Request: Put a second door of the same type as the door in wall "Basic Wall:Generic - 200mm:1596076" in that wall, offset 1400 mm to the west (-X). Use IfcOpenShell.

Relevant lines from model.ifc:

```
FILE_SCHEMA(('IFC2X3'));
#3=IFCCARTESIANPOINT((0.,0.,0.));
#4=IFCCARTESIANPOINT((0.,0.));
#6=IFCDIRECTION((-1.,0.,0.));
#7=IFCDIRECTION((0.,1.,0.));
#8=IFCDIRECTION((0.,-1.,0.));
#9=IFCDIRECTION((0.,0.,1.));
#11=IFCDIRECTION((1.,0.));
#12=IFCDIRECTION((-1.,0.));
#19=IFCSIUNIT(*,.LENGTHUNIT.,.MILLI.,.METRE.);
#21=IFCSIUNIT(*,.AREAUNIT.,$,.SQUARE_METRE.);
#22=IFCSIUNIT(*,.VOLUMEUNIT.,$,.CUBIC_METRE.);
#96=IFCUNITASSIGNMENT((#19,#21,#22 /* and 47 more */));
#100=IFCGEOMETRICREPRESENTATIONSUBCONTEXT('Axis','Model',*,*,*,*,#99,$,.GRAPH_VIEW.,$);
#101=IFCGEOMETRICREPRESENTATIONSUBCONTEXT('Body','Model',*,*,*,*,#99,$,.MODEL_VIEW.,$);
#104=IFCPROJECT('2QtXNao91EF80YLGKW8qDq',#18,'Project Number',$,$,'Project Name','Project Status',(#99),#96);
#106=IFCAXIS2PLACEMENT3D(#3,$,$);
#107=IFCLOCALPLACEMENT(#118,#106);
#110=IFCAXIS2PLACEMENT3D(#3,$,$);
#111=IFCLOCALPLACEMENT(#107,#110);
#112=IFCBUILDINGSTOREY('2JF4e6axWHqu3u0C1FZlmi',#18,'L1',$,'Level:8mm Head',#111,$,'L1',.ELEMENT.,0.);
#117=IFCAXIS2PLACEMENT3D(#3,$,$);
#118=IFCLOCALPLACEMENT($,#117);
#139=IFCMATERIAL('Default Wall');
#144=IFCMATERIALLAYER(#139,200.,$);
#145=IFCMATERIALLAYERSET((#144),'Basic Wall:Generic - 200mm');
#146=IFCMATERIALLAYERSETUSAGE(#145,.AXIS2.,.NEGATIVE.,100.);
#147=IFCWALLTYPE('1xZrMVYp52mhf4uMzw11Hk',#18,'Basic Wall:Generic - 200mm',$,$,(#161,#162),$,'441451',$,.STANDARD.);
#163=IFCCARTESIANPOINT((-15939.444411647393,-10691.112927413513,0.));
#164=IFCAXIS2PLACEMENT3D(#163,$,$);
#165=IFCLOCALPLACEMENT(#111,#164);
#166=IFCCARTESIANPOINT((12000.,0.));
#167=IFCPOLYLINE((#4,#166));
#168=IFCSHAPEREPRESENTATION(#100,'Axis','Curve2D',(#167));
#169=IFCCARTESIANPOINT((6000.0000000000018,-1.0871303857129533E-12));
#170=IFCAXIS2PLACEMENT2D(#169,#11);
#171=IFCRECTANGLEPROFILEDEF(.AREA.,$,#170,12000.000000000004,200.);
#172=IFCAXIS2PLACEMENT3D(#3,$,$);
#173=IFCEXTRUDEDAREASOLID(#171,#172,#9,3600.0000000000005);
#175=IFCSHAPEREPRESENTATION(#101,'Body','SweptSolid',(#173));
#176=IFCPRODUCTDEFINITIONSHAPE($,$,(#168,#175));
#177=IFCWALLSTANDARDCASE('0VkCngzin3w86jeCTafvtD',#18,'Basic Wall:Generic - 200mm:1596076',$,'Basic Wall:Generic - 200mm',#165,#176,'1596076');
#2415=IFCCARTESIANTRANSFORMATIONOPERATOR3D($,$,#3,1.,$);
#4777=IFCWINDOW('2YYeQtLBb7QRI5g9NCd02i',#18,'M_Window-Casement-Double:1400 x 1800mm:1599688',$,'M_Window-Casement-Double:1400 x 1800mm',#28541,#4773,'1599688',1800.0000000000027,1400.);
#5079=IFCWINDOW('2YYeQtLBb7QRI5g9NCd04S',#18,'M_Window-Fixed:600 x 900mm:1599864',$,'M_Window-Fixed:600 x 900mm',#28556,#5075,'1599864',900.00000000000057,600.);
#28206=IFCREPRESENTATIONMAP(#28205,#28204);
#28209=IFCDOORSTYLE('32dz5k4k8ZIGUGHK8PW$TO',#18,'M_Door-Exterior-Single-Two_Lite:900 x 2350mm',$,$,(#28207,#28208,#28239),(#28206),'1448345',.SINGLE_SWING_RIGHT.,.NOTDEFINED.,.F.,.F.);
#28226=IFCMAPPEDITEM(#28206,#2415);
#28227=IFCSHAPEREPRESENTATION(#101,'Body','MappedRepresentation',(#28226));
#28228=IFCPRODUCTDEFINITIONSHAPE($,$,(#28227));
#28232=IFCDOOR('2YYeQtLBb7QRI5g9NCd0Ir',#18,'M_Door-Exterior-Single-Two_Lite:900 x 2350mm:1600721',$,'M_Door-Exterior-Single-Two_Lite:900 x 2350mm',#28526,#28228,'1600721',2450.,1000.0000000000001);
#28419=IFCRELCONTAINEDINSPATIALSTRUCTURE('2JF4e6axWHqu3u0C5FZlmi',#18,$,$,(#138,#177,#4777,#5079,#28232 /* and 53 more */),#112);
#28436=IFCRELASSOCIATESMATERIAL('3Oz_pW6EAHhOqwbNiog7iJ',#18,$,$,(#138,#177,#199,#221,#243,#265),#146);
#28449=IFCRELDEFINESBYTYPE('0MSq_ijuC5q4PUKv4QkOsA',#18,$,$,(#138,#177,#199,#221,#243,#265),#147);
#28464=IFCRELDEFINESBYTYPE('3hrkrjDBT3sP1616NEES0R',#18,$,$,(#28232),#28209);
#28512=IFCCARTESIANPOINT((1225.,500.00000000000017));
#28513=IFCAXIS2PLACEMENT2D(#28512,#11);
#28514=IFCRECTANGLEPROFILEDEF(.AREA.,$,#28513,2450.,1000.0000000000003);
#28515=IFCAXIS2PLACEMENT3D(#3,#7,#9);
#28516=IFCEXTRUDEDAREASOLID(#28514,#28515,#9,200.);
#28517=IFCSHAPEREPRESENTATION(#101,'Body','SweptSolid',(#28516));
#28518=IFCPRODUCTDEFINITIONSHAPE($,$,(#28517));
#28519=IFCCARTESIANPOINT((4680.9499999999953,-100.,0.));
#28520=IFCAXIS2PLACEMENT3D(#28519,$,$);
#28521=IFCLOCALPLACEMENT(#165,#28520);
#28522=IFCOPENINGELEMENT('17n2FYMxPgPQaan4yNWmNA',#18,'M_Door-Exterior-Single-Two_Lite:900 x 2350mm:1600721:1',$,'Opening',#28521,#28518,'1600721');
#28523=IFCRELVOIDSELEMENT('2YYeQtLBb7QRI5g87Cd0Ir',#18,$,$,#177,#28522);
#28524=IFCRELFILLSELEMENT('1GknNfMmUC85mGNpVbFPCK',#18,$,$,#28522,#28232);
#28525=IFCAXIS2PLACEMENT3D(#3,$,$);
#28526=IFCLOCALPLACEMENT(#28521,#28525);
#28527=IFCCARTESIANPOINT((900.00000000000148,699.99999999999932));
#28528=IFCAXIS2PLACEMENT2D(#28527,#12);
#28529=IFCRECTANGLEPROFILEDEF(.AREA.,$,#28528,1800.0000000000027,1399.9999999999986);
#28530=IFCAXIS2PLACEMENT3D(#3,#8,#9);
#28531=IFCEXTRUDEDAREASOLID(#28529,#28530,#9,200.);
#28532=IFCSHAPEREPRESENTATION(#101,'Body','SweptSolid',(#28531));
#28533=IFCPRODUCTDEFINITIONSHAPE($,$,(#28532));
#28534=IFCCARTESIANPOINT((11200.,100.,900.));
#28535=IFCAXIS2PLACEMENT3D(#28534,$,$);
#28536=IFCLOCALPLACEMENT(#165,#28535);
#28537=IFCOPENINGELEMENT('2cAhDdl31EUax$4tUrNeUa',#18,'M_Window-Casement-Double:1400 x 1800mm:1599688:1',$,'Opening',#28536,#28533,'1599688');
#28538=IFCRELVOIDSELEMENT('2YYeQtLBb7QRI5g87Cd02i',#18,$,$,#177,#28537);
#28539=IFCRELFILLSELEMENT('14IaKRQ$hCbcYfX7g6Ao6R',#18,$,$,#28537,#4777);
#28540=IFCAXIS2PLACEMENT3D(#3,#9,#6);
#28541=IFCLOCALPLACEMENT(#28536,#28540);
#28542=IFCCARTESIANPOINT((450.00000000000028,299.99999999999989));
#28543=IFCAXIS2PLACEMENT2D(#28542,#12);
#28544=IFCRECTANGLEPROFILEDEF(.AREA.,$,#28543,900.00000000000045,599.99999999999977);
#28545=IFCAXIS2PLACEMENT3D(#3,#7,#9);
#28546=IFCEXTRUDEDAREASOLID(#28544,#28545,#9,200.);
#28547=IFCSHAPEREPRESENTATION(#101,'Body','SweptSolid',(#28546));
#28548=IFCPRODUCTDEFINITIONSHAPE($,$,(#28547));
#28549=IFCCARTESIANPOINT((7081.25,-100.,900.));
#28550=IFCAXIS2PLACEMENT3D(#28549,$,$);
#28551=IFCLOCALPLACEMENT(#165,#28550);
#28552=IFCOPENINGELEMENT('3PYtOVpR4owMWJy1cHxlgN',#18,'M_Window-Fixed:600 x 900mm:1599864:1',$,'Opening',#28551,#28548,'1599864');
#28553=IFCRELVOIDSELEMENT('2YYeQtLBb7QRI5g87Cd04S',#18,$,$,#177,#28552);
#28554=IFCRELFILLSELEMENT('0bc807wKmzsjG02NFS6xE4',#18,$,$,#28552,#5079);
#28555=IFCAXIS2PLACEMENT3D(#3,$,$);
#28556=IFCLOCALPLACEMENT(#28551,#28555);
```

```python
import ifcopenshell
import ifcopenshell.api.feature
import ifcopenshell.api.geometry
import ifcopenshell.api.root
import ifcopenshell.geom
import ifcopenshell.util.element
import ifcopenshell.util.placement
import ifcopenshell.util.shape

model = ifcopenshell.open("model.ifc")
settings = ifcopenshell.geom.settings()


def volume(element):
    """Net volume in cubic metres, openings subtracted."""
    shape = ifcopenshell.geom.create_shape(settings, element)
    return ifcopenshell.util.shape.get_volume(shape.geometry)


def reuse_history(source, copy):
    """copy_class also copies each property set's owner history, people and application; keep the originals."""
    for rel in copy.IsDefinedBy:
        if rel.is_a("IfcRelDefinesByProperties") and (history := rel.RelatingPropertyDefinition.OwnerHistory):
            rel.RelatingPropertyDefinition.OwnerHistory = source.OwnerHistory
            ifcopenshell.util.element.remove_deep2(model, history)


door = model.by_guid("2YYeQtLBb7QRI5g9NCd0Ir")
opening = door.FillsVoids[0].RelatingOpeningElement
wall = opening.VoidsElements[0].RelatingBuildingElement
before = volume(wall)
shift = ifcopenshell.util.placement.get_local_placement(wall.ObjectPlacement)[:3, 0] * -1400.0

# copy_class copies the void relationship, type, container and properties, but no geometry.
new_opening = ifcopenshell.api.root.copy_class(model, product=opening)
new_opening.Representation = ifcopenshell.util.element.copy_deep(
    model, opening.Representation, exclude=["IfcGeometricRepresentationContext", "IfcRepresentationMap"]
)
new_opening.Name = "M_Door-Exterior-Single-Two_Lite:900 x 2350mm"
new_opening.Tag = None
new_door = ifcopenshell.api.root.copy_class(model, product=door)
new_door.Representation = ifcopenshell.util.element.copy_deep(
    model, door.Representation, exclude=["IfcGeometricRepresentationContext", "IfcRepresentationMap"]
)
new_door.Name = "M_Door-Exterior-Single-Two_Lite:900 x 2350mm"
new_door.Tag = None
reuse_history(door, new_door)
fills = ifcopenshell.api.feature.add_filling(model, opening=new_opening, element=new_door)
fills.OwnerHistory = new_door.OwnerHistory  # required in IFC2X3

for old, new in ((opening, new_opening), (door, new_door)):
    matrix = ifcopenshell.util.placement.get_local_placement(old.ObjectPlacement)
    matrix[:3, 3] += shift
    ifcopenshell.api.geometry.edit_object_placement(model, product=new, matrix=matrix, is_si=False)

after = volume(wall)

print(f"wall volume {before:.3f} -> {after:.3f} m3")

model.write("model_rev.ifc")
```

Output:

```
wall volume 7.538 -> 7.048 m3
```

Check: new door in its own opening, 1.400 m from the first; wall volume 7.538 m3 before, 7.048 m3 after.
